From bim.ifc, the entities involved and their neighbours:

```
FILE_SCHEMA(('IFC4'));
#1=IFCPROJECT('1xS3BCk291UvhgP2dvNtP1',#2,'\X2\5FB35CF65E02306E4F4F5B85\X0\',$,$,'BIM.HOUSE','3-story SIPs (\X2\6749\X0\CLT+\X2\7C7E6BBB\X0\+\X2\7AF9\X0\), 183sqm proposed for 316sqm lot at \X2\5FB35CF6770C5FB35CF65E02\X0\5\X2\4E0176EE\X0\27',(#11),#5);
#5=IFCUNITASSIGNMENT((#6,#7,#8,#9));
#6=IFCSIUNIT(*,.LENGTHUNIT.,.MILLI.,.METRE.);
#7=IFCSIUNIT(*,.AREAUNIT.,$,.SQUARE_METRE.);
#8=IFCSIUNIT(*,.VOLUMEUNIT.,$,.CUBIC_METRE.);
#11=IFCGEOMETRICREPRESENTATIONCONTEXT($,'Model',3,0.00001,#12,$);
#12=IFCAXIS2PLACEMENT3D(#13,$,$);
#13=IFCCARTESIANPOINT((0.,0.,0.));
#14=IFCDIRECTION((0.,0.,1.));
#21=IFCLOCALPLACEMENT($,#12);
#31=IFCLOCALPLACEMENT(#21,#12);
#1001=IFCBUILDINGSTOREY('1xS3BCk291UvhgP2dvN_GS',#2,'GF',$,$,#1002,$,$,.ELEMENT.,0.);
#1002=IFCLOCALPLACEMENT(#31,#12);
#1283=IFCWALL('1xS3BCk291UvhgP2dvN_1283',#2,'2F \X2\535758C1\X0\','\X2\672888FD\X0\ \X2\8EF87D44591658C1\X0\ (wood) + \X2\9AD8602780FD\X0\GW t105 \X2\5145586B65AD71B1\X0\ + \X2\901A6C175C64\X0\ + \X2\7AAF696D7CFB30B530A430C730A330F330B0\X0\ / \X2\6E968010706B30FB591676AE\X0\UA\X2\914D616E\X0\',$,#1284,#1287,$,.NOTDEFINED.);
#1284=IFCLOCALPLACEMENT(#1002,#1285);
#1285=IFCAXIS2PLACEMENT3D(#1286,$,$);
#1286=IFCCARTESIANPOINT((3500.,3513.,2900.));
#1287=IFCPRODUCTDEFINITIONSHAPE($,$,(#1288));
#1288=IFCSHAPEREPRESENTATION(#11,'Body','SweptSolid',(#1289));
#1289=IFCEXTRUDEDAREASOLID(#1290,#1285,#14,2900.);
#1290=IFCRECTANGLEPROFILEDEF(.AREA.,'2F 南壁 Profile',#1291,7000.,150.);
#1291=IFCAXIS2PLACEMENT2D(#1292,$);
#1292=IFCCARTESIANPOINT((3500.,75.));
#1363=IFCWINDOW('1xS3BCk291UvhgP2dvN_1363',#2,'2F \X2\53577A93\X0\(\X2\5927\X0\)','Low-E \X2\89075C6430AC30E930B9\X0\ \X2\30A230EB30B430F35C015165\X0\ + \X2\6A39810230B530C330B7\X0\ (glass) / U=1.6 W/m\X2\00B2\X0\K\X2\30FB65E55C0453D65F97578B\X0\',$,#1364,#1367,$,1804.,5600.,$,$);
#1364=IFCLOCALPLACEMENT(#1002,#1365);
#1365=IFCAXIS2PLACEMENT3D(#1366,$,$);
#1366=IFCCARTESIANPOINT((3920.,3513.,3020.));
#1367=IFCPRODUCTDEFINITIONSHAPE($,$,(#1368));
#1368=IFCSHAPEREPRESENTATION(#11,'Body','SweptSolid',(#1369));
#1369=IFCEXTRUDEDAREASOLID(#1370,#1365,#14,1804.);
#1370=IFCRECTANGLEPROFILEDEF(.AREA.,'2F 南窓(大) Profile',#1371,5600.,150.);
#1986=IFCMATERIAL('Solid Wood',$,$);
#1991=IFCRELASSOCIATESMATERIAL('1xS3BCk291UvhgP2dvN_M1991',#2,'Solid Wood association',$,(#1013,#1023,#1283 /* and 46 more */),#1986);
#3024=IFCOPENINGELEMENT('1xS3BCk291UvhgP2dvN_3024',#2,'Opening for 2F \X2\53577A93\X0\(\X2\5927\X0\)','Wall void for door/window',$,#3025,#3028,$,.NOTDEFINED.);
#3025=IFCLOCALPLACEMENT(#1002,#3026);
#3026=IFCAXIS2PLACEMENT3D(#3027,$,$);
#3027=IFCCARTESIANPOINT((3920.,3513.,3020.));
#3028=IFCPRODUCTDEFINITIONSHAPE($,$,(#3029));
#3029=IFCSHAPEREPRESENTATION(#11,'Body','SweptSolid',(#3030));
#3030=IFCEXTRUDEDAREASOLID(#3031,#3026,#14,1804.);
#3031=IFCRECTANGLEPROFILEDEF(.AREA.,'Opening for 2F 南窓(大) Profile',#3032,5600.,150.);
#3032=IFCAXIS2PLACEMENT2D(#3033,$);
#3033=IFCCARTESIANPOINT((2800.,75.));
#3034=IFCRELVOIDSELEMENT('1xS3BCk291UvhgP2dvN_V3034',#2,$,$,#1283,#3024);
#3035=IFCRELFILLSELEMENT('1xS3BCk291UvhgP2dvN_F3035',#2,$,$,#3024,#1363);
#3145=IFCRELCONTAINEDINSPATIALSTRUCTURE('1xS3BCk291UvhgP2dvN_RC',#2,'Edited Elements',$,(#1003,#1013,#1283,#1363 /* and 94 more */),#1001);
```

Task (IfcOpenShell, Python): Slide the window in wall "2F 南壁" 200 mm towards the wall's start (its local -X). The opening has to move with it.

```python
import ifcopenshell
import ifcopenshell.api.geometry
import ifcopenshell.util.placement
import ifcopenshell.util.unit

model = ifcopenshell.open("bim.ifc")
unit_scale = ifcopenshell.util.unit.calculate_unit_scale(model)

window = model.by_guid("1xS3BCk291UvhgP2dvN_1363")
opening = window.FillsVoids[0].RelatingOpeningElement
wall = opening.VoidsElements[0].RelatingBuildingElement

wall_matrix = ifcopenshell.util.placement.get_local_placement(wall.ObjectPlacement)
shift = wall_matrix[:3, 0] * -0.2 / unit_scale
before = ifcopenshell.util.placement.get_local_placement(window.ObjectPlacement)[:3, 3].copy()

# The window is not placed relative to its opening, so move both.
for product in (opening, window):
    matrix = ifcopenshell.util.placement.get_local_placement(product.ObjectPlacement)
    matrix[:3, 3] += shift
    ifcopenshell.api.geometry.edit_object_placement(model, product=product, matrix=matrix, is_si=False)

after = ifcopenshell.util.placement.get_local_placement(window.ObjectPlacement)[:3, 3]
print("window moved by", (after - before).round(3) + 0.0)

model.write("bim_rev.ifc")
```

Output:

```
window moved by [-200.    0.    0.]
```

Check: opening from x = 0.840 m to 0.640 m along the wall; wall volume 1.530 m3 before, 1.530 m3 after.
